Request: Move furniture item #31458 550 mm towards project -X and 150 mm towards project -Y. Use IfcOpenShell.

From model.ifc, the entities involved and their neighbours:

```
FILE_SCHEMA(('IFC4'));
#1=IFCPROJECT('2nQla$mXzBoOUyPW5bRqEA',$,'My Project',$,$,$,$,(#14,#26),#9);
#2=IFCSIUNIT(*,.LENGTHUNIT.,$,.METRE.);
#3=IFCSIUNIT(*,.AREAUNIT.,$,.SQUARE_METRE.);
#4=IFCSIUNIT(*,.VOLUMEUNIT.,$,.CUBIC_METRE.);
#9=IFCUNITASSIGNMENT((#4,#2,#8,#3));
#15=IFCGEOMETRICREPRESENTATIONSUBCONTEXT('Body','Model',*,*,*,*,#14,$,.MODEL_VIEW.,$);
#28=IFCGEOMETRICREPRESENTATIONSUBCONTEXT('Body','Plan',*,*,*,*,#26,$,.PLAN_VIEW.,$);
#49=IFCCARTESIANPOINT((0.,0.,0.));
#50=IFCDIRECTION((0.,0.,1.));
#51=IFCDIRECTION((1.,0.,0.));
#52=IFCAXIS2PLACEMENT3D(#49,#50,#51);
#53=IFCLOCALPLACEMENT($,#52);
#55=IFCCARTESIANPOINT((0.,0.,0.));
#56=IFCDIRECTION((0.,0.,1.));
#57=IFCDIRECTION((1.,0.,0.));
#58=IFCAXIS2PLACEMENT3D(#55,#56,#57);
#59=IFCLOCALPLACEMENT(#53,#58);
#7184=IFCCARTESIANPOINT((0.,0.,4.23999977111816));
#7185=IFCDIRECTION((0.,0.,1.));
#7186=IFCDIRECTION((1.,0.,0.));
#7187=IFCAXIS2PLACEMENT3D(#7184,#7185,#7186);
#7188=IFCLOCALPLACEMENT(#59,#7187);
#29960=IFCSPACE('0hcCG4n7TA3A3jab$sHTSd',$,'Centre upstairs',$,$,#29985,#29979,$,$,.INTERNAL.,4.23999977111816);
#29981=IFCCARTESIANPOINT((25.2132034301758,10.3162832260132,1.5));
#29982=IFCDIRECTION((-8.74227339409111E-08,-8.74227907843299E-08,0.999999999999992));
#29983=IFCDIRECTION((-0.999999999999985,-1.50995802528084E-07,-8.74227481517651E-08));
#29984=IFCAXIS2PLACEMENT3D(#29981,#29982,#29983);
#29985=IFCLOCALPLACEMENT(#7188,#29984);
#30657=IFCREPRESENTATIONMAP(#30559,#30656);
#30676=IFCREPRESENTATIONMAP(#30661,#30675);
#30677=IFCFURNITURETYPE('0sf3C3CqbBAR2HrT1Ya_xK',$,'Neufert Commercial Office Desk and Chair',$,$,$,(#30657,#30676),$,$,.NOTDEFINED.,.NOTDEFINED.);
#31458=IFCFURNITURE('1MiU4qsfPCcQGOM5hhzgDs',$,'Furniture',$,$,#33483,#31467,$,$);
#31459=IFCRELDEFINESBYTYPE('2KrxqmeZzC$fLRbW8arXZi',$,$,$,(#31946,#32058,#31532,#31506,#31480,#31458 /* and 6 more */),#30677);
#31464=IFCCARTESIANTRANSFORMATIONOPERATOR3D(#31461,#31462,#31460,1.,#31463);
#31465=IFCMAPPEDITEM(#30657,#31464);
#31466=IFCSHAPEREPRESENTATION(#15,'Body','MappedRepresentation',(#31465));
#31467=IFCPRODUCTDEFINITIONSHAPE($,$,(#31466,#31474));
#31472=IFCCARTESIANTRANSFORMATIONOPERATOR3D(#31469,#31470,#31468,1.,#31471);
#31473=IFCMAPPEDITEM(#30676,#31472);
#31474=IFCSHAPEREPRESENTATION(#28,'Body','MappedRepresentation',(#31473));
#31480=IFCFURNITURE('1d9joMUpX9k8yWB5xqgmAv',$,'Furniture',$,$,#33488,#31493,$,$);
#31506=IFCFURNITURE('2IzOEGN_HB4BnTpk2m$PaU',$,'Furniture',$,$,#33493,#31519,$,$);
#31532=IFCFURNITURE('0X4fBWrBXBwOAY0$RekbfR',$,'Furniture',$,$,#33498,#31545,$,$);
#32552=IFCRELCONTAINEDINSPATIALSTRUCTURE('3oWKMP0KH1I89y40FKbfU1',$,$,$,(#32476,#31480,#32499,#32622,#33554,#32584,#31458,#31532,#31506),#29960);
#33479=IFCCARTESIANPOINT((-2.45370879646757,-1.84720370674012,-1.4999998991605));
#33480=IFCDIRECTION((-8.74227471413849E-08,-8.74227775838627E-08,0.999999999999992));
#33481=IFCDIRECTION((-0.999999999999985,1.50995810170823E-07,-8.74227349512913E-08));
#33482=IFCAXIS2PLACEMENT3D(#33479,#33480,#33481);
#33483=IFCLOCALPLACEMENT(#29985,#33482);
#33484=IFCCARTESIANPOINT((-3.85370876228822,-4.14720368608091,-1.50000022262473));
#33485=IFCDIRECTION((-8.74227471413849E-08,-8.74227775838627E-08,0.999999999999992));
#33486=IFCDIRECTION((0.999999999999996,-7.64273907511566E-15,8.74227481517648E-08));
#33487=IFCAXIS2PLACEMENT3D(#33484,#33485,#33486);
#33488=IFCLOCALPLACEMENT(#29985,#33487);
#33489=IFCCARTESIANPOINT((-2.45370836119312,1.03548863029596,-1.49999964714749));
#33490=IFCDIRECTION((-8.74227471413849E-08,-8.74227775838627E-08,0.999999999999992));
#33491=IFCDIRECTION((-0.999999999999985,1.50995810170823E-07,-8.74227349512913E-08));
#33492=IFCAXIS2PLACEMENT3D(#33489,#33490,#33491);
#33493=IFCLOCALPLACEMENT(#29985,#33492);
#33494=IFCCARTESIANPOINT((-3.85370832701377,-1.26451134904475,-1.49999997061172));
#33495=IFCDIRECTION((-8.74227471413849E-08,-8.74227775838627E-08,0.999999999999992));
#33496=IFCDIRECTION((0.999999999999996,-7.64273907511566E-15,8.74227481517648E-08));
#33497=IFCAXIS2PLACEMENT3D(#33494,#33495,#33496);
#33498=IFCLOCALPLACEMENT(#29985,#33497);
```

```python
import ifcopenshell
import ifcopenshell.api.geometry
import ifcopenshell.util.placement
import ifcopenshell.util.unit

model = ifcopenshell.open("model.ifc")
unit_scale = ifcopenshell.util.unit.calculate_unit_scale(model)

item = model.by_id(31458)
matrix = ifcopenshell.util.placement.get_local_placement(item.ObjectPlacement)
matrix[0, 3] -= 0.55 / unit_scale
matrix[1, 3] -= 0.15 / unit_scale
ifcopenshell.api.geometry.edit_object_placement(model, product=item, matrix=matrix, is_si=False)

print(ifcopenshell.util.placement.get_local_placement(item.ObjectPlacement).round(3) + 0.0)

model.write("model_rev.ifc")
```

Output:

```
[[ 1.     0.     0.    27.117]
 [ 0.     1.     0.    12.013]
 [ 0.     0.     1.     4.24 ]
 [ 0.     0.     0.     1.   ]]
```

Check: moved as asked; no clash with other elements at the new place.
